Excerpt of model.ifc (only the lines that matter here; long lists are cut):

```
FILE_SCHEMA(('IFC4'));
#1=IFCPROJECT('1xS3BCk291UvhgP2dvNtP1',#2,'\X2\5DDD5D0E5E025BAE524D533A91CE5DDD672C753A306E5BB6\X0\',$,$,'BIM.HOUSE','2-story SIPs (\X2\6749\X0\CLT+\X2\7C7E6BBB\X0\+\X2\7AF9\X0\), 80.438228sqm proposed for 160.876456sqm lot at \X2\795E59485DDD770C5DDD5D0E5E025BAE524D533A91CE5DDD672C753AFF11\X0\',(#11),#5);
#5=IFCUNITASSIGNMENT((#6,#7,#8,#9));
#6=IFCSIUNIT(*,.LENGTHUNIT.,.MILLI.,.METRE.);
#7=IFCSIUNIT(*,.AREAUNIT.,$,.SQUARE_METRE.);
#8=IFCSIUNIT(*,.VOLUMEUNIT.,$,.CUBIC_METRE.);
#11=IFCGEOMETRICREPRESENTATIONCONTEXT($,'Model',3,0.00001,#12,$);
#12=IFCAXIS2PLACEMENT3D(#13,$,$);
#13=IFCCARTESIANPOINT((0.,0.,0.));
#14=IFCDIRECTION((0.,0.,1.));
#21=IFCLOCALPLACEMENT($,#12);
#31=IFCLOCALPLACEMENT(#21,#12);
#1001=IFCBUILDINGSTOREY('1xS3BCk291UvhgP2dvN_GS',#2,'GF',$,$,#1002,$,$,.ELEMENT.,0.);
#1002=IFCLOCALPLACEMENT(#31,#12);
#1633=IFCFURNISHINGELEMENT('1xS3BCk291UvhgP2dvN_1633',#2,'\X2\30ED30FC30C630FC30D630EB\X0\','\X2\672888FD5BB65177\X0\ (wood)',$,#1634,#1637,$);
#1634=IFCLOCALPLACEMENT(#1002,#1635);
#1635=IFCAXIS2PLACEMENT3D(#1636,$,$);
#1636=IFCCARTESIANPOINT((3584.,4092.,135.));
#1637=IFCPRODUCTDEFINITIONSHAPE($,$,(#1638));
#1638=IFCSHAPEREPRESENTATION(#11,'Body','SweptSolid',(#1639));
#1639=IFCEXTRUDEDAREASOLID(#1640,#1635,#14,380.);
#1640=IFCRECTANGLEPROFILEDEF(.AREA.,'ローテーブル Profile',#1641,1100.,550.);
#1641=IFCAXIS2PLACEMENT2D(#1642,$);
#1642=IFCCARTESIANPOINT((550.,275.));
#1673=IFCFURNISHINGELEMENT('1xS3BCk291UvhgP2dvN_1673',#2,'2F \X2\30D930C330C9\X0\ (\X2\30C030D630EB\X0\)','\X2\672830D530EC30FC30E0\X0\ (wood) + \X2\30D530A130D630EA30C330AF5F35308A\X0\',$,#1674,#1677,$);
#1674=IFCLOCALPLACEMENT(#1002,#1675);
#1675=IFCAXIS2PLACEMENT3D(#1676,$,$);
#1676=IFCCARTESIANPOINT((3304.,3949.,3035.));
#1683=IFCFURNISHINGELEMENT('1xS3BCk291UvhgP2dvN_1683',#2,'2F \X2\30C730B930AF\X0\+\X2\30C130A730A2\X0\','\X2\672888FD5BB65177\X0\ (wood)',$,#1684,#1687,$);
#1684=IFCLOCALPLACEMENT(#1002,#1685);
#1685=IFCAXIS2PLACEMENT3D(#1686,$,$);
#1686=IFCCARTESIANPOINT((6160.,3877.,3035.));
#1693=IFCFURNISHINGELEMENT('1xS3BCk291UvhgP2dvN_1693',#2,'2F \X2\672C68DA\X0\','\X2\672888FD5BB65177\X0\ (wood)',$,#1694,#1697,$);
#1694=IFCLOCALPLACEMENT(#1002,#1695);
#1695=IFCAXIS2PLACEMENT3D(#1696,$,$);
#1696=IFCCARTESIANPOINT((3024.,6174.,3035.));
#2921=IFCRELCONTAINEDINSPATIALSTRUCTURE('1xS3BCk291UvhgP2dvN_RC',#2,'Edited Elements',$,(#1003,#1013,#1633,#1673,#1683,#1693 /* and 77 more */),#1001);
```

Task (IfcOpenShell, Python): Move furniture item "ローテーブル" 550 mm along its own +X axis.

```python
import ifcopenshell
import ifcopenshell.api.geometry
import ifcopenshell.util.placement

model = ifcopenshell.open("model.ifc")

item = model.by_guid("1xS3BCk291UvhgP2dvN_1633")
matrix = ifcopenshell.util.placement.get_local_placement(item.ObjectPlacement)
matrix[:3, 3] += matrix[:3, 0] * 550.0
ifcopenshell.api.geometry.edit_object_placement(model, product=item, matrix=matrix, is_si=False)

print(ifcopenshell.util.placement.get_local_placement(item.ObjectPlacement).round(3) + 0.0)

model.write("model-out.ifc")
```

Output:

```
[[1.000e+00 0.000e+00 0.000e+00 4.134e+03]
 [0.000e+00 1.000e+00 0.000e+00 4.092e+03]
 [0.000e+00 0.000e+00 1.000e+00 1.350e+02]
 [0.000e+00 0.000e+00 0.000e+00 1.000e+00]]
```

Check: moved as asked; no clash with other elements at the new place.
